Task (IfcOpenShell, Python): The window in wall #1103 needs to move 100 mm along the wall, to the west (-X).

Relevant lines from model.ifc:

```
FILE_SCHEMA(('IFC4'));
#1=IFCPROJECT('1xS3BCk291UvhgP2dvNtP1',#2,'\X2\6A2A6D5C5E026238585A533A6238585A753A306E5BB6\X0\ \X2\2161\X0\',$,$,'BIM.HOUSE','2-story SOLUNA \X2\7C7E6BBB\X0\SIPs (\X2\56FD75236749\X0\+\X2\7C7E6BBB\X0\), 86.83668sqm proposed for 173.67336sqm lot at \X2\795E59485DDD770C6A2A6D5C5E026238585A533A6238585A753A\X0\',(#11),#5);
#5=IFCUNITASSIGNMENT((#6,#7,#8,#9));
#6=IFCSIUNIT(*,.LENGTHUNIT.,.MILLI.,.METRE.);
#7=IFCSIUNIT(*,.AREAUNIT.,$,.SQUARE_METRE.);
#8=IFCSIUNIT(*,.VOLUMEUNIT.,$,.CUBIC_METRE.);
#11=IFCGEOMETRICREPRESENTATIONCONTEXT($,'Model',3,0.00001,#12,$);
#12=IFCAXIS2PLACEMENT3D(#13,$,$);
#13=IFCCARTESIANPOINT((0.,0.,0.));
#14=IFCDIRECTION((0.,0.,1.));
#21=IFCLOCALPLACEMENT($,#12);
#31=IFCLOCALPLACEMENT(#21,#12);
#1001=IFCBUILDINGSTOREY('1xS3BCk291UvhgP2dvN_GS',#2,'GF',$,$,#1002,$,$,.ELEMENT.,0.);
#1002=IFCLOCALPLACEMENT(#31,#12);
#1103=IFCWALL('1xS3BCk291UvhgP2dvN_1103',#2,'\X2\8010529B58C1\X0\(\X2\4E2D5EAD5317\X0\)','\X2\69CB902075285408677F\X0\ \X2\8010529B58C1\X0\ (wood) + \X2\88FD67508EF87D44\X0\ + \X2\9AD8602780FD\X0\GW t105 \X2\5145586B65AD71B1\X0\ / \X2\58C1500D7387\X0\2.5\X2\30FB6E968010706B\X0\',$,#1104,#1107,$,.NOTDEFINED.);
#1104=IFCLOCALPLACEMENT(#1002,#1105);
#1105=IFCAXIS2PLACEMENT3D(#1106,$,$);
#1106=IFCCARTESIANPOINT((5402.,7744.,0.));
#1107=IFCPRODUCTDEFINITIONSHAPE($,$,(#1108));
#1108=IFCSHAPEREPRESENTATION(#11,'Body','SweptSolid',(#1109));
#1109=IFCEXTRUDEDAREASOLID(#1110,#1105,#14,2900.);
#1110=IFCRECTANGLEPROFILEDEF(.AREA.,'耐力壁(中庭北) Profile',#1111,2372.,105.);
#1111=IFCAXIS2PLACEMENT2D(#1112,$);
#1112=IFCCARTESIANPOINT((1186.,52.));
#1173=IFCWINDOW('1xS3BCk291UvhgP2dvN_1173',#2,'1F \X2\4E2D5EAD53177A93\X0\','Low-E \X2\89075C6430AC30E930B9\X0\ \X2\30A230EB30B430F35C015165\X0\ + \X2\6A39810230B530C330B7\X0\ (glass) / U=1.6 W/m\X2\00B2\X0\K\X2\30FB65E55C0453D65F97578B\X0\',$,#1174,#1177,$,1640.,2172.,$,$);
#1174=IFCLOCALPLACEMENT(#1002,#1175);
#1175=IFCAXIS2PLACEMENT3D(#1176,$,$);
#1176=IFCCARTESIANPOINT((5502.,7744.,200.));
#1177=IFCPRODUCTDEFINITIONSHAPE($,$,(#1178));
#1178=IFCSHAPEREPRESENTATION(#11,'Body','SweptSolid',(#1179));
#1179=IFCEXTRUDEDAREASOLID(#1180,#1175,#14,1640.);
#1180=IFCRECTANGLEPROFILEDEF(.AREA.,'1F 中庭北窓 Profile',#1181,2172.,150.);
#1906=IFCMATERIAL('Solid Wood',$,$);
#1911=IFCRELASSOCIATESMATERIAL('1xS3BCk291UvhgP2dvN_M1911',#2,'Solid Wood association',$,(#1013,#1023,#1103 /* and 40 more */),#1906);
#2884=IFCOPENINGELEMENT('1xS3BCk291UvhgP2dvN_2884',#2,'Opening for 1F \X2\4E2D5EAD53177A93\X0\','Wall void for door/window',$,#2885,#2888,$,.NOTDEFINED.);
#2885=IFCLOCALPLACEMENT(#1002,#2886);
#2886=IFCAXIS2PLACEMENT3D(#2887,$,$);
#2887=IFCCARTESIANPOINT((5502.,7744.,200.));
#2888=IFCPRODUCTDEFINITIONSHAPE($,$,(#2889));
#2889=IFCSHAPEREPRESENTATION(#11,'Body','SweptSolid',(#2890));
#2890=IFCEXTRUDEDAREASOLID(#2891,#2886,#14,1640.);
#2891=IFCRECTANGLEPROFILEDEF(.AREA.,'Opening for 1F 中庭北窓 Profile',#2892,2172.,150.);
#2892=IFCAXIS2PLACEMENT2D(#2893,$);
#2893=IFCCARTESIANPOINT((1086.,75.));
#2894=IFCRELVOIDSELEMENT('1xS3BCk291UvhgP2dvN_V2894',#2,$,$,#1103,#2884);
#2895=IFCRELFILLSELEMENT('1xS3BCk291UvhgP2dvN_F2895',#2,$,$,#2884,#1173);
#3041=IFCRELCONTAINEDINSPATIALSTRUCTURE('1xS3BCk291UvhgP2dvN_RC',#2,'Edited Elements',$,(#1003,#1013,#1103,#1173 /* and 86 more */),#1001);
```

```python
import ifcopenshell
import ifcopenshell.api.geometry
import ifcopenshell.util.placement
import ifcopenshell.util.unit

model = ifcopenshell.open("model.ifc")
unit_scale = ifcopenshell.util.unit.calculate_unit_scale(model)

window = model.by_guid("1xS3BCk291UvhgP2dvN_1173")
opening = window.FillsVoids[0].RelatingOpeningElement
wall = opening.VoidsElements[0].RelatingBuildingElement

wall_matrix = ifcopenshell.util.placement.get_local_placement(wall.ObjectPlacement)
shift = wall_matrix[:3, 0] * -0.1 / unit_scale
before = ifcopenshell.util.placement.get_local_placement(window.ObjectPlacement)[:3, 3].copy()

# The window is not placed relative to its opening, so move both.
for product in (opening, window):
    matrix = ifcopenshell.util.placement.get_local_placement(product.ObjectPlacement)
    matrix[:3, 3] += shift
    ifcopenshell.api.geometry.edit_object_placement(model, product=product, matrix=matrix, is_si=False)

after = ifcopenshell.util.placement.get_local_placement(window.ObjectPlacement)[:3, 3]
print("window moved by", (after - before).round(3) + 0.0)

model.write("model_edited.ifc")
```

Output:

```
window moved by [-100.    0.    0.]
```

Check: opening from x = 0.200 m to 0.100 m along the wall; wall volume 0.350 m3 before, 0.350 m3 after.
